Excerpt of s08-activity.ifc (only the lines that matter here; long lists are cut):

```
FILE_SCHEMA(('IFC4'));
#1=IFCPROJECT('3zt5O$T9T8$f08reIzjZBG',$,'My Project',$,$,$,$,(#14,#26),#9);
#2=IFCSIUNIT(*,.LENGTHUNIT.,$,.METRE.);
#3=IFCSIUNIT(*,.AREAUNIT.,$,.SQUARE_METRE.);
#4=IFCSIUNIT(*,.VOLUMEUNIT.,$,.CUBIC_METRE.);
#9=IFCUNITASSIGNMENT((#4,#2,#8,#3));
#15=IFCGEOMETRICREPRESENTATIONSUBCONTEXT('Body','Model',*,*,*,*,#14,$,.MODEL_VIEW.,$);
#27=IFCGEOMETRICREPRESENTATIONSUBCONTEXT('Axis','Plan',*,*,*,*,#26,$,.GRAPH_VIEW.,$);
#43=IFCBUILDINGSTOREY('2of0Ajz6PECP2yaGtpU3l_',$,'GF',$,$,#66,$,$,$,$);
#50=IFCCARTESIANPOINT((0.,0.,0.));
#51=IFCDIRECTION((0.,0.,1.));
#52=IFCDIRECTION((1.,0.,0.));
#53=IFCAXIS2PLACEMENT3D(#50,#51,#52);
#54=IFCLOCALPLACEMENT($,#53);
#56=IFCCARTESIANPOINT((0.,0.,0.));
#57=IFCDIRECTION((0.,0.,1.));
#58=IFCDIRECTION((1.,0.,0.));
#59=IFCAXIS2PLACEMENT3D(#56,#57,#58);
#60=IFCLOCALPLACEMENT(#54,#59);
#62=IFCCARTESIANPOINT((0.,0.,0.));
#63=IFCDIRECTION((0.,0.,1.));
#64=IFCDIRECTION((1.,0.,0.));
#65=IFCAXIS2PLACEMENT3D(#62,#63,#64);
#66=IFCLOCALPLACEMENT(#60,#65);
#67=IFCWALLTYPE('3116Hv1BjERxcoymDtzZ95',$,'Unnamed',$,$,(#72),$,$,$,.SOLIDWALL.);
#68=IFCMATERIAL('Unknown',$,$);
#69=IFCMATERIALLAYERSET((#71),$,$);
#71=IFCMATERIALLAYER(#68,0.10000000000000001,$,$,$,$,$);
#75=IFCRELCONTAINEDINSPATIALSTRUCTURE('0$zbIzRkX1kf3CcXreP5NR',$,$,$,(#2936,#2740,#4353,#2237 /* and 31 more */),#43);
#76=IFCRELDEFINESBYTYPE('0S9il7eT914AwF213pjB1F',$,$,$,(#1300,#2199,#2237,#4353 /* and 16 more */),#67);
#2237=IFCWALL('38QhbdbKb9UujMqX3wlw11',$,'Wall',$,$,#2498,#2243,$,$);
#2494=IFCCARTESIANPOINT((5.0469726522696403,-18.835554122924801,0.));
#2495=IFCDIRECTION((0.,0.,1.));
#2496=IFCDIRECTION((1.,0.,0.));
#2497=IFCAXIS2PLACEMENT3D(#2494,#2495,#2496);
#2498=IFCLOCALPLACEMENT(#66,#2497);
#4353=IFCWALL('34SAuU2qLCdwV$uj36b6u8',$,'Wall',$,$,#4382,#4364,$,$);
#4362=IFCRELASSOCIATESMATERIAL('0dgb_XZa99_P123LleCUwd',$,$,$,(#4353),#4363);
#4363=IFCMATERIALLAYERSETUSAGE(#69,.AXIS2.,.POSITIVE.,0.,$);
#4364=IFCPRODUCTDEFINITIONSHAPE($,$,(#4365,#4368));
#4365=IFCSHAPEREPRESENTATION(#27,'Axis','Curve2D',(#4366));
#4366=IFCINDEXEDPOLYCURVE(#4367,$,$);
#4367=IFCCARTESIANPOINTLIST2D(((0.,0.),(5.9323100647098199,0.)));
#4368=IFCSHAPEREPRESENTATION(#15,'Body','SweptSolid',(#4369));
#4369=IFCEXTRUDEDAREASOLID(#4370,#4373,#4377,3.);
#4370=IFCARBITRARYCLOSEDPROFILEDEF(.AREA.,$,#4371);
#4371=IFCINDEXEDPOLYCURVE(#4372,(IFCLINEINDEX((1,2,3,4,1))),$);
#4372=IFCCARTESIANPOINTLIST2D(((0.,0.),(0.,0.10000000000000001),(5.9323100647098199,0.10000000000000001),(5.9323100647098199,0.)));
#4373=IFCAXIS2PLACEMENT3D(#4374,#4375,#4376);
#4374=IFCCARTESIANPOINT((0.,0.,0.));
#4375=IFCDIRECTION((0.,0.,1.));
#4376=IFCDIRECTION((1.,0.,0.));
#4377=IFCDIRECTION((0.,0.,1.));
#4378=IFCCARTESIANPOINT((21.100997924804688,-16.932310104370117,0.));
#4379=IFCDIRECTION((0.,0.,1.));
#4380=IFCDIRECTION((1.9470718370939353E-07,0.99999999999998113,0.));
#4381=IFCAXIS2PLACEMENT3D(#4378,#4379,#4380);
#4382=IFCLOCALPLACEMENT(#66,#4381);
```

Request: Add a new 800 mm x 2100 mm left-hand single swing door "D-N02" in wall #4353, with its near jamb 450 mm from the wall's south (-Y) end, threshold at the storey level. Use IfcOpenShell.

```python
import numpy as np
import ifcopenshell
import ifcopenshell.api.feature
import ifcopenshell.api.geometry
import ifcopenshell.api.root
import ifcopenshell.api.spatial
import ifcopenshell.geom
import ifcopenshell.util.element
import ifcopenshell.util.placement
import ifcopenshell.util.representation
import ifcopenshell.util.shape
import ifcopenshell.util.unit

model = ifcopenshell.open("s08-activity.ifc")
unit_scale = ifcopenshell.util.unit.calculate_unit_scale(model)
settings = ifcopenshell.geom.settings()


def volume(element):
    """Net volume in cubic metres, openings subtracted."""
    shape = ifcopenshell.geom.create_shape(settings, element)
    return ifcopenshell.util.shape.get_volume(shape.geometry)


wall = model.by_guid("34SAuU2qLCdwV$uj36b6u8")
storey = ifcopenshell.util.element.get_container(wall, ifc_class="IfcBuildingStorey")
context = ifcopenshell.util.representation.get_context(model, "Model", "Body", "MODEL_VIEW")
before = volume(wall)

width, height, from_end, sill = 0.8, 2.1, 0.45, 0.0  # metres

# The wall runs along its own X axis, and the end named is its -X end.
wall_shape = ifcopenshell.geom.create_shape(settings, wall)
x, y, z = ifcopenshell.util.shape.get_vertices(wall_shape.geometry).T
start = x.min() + from_end
face, thickness = float(y.min()), float(y.max() - y.min())
wall_matrix = ifcopenshell.util.placement.get_local_placement(wall.ObjectPlacement)
level = ifcopenshell.util.placement.get_local_placement(storey.ObjectPlacement)[2, 3]


def in_wall(x, y):
    """Placement at x, y metres in the wall's axes, at sill height."""
    matrix = wall_matrix.copy()
    matrix[:, 3] = wall_matrix @ np.array([x / unit_scale, y / unit_scale, 0.0, 1.0])
    matrix[2, 3] = level + sill / unit_scale
    return matrix


# Opening: a box that overshoots both wall faces by 50 mm.
opening = ifcopenshell.api.root.create_entity(model, ifc_class="IfcOpeningElement", predefined_type="OPENING")
box = ifcopenshell.api.geometry.add_wall_representation(
    model, context=context, length=width, height=height, thickness=thickness + 0.1
)
ifcopenshell.api.geometry.assign_representation(model, product=opening, representation=box)
ifcopenshell.api.geometry.edit_object_placement(model, product=opening, matrix=in_wall(start, face - 0.05), is_si=False)
ifcopenshell.api.feature.add_feature(model, feature=opening, element=wall)

door = ifcopenshell.api.root.create_entity(model, ifc_class="IfcDoor", name="D-N02", predefined_type="DOOR")
door.OverallWidth, door.OverallHeight = width / unit_scale, height / unit_scale
door.OperationType = "SINGLE_SWING_LEFT"
body = ifcopenshell.api.geometry.add_door_representation(
    model,
    context=context,
    overall_width=door.OverallWidth,
    overall_height=door.OverallHeight,
    operation_type="SINGLE_SWING_LEFT",
    lining_properties={"LiningDepth": thickness / unit_scale, "ThresholdDepth": thickness / unit_scale},
)
ifcopenshell.api.geometry.assign_representation(model, product=door, representation=body)
ifcopenshell.api.spatial.assign_container(model, products=[door], relating_structure=storey)
ifcopenshell.api.feature.add_filling(model, opening=opening, element=door)

# The lining spans the wall, so the door starts at the wall face.
ifcopenshell.api.geometry.edit_object_placement(model, product=door, matrix=in_wall(start, face), is_si=False)

after = volume(wall)

print(f"wall volume {before:.3f} -> {after:.3f} m3")

model.write("s08-activity-out.ifc")
```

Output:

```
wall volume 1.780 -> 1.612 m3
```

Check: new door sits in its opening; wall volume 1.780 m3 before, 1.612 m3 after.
